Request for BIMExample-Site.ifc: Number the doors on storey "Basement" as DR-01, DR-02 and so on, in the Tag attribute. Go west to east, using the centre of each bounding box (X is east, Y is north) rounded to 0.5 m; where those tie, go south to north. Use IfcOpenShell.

First a look at what the model holds.

```python
import ifcopenshell
import ifcopenshell.util.element
import ifcopenshell.util.placement

model = ifcopenshell.open("BIMExample-Site.ifc")
print(model.schema)
storey = next(s for s in model.by_type("IfcBuildingStorey") if s.Name == "Basement")
doors = [e for e in ifcopenshell.util.element.get_decomposition(storey) if e.is_a("IfcDoor")]
for e in sorted(doors, key=lambda e: e.id()):
    origin = ifcopenshell.util.placement.get_local_placement(e.ObjectPlacement)[:3, 3]
    print(e.id(), e.Tag, e.Name, origin.round(2) + 0.0, sep=" | ")
```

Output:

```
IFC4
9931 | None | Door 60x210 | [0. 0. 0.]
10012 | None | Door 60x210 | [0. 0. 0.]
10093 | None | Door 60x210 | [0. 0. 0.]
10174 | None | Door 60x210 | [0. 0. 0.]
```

```python
import ifcopenshell
import ifcopenshell.geom
import ifcopenshell.util.element
import ifcopenshell.util.shape

model = ifcopenshell.open("BIMExample-Site.ifc")
settings = ifcopenshell.geom.settings()
settings.set("use-world-coords", True)


def centre(element):
    shape = ifcopenshell.geom.create_shape(settings, element)
    return ifcopenshell.util.shape.get_bbox_centroid(shape.geometry)


storey = next(s for s in model.by_type("IfcBuildingStorey") if s.Name == "Basement")
doors = [e for e in ifcopenshell.util.element.get_decomposition(storey) if e.is_a("IfcDoor")]

# Insertion points can sit at a corner or the storey origin, so sort by the geometry (in metres).
centres = {e: centre(e) for e in doors}
doors.sort(key=lambda e: (round(centres[e][0] / 0.5), centres[e][1]))

for i, e in enumerate(doors, start=1):
    number = f"DR-{i:02d}"
    e.Tag = number
    print(e.id(), number)

model.write("BIMExample-Site-out.ifc")
```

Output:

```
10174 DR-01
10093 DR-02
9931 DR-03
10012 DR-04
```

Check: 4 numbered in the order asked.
